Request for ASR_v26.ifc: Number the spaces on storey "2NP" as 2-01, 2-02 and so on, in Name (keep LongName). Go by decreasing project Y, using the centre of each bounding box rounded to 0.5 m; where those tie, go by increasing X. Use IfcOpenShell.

First a look at what the model holds.

```python
import ifcopenshell
import ifcopenshell.util.element
import ifcopenshell.util.placement

model = ifcopenshell.open("ASR_v26.ifc")
print(model.schema)
storey = next(s for s in model.by_type("IfcBuildingStorey") if s.Name == "2NP")
spaces = [e for e in ifcopenshell.util.element.get_decomposition(storey) if e.is_a("IfcSpace")]
for e in sorted(spaces, key=lambda e: e.id()):
    origin = ifcopenshell.util.placement.get_local_placement(e.ObjectPlacement)[:3, 3]
    print(e.id(), e.Name, e.LongName, origin.round(2) + 0.0, sep=" | ")
```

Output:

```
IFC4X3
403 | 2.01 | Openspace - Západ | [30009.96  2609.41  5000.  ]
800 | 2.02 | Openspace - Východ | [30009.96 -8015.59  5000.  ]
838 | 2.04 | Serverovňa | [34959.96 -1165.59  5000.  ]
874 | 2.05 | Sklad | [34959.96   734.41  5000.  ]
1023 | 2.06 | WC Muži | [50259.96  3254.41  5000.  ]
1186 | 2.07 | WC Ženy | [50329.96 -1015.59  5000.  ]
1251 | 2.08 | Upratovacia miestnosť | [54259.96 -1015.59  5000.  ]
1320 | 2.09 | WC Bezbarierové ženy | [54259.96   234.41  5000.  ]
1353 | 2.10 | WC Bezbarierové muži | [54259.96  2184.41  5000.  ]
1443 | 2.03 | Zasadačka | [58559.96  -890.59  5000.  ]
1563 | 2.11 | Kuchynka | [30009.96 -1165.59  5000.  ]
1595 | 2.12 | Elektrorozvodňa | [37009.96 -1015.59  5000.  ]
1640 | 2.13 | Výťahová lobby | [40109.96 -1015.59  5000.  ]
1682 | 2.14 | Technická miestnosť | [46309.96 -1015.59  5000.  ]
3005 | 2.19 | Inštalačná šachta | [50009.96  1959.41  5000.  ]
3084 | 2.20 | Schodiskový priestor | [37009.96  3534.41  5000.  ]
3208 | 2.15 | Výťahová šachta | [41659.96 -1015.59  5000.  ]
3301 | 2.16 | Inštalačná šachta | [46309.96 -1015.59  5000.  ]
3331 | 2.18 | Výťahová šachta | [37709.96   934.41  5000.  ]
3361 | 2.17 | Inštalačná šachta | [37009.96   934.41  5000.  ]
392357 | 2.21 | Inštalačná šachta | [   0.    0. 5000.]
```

```python
import ifcopenshell
import ifcopenshell.geom
import ifcopenshell.util.element
import ifcopenshell.util.shape

model = ifcopenshell.open("ASR_v26.ifc")
settings = ifcopenshell.geom.settings()
settings.set("use-world-coords", True)


def centre(element):
    shape = ifcopenshell.geom.create_shape(settings, element)
    return ifcopenshell.util.shape.get_bbox_centroid(shape.geometry)


storey = next(s for s in model.by_type("IfcBuildingStorey") if s.Name == "2NP")
spaces = [e for e in ifcopenshell.util.element.get_decomposition(storey) if e.is_a("IfcSpace")]

# Insertion points can sit at a corner or the storey origin, so sort by the geometry (in metres).
centres = {e: centre(e) for e in spaces}
spaces.sort(key=lambda e: (-round(centres[e][1] / 0.5), centres[e][0]))

for i, e in enumerate(spaces, start=1):
    number = f"2-{i:02d}"
    e.Name = number
    print(e.id(), number)

model.write("ASR_v26_rev.ifc")
```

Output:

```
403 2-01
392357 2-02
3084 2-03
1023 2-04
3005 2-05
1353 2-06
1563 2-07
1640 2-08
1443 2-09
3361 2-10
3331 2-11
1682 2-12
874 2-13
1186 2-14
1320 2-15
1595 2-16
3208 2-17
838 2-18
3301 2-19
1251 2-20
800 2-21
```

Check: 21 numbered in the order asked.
